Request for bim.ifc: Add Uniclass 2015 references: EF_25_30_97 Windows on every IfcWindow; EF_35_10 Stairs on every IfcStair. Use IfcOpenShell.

First a look at what the model holds.

```python
import ifcopenshell

model = ifcopenshell.open("bim.ifc")
print(model.schema)
print("classifications:", [c.Name for c in model.by_type("IfcClassification")])
for ifc_class in ("IfcDoor", "IfcRoof", "IfcStair", "IfcWall", "IfcWindow"):
    print(ifc_class, len(model.by_type(ifc_class)))
```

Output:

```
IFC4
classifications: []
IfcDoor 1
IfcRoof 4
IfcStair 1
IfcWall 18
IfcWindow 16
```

```python
import ifcopenshell
import ifcopenshell.api.classification

model = ifcopenshell.open("bim.ifc")

system = ifcopenshell.api.classification.add_classification(model, classification="Uniclass 2015")

codes = {
    "IfcWindow": ("EF_25_30_97", "Windows"),
    "IfcStair": ("EF_35_10", "Stairs"),
}
for ifc_class, (code, name) in codes.items():
    products = model.by_type(ifc_class)
    ifcopenshell.api.classification.add_reference(
        model, products=products, classification=system, identification=code, name=name
    )
    print(code, len(products))

model.write("bim-out.ifc")
```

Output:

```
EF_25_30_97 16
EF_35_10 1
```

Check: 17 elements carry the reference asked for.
